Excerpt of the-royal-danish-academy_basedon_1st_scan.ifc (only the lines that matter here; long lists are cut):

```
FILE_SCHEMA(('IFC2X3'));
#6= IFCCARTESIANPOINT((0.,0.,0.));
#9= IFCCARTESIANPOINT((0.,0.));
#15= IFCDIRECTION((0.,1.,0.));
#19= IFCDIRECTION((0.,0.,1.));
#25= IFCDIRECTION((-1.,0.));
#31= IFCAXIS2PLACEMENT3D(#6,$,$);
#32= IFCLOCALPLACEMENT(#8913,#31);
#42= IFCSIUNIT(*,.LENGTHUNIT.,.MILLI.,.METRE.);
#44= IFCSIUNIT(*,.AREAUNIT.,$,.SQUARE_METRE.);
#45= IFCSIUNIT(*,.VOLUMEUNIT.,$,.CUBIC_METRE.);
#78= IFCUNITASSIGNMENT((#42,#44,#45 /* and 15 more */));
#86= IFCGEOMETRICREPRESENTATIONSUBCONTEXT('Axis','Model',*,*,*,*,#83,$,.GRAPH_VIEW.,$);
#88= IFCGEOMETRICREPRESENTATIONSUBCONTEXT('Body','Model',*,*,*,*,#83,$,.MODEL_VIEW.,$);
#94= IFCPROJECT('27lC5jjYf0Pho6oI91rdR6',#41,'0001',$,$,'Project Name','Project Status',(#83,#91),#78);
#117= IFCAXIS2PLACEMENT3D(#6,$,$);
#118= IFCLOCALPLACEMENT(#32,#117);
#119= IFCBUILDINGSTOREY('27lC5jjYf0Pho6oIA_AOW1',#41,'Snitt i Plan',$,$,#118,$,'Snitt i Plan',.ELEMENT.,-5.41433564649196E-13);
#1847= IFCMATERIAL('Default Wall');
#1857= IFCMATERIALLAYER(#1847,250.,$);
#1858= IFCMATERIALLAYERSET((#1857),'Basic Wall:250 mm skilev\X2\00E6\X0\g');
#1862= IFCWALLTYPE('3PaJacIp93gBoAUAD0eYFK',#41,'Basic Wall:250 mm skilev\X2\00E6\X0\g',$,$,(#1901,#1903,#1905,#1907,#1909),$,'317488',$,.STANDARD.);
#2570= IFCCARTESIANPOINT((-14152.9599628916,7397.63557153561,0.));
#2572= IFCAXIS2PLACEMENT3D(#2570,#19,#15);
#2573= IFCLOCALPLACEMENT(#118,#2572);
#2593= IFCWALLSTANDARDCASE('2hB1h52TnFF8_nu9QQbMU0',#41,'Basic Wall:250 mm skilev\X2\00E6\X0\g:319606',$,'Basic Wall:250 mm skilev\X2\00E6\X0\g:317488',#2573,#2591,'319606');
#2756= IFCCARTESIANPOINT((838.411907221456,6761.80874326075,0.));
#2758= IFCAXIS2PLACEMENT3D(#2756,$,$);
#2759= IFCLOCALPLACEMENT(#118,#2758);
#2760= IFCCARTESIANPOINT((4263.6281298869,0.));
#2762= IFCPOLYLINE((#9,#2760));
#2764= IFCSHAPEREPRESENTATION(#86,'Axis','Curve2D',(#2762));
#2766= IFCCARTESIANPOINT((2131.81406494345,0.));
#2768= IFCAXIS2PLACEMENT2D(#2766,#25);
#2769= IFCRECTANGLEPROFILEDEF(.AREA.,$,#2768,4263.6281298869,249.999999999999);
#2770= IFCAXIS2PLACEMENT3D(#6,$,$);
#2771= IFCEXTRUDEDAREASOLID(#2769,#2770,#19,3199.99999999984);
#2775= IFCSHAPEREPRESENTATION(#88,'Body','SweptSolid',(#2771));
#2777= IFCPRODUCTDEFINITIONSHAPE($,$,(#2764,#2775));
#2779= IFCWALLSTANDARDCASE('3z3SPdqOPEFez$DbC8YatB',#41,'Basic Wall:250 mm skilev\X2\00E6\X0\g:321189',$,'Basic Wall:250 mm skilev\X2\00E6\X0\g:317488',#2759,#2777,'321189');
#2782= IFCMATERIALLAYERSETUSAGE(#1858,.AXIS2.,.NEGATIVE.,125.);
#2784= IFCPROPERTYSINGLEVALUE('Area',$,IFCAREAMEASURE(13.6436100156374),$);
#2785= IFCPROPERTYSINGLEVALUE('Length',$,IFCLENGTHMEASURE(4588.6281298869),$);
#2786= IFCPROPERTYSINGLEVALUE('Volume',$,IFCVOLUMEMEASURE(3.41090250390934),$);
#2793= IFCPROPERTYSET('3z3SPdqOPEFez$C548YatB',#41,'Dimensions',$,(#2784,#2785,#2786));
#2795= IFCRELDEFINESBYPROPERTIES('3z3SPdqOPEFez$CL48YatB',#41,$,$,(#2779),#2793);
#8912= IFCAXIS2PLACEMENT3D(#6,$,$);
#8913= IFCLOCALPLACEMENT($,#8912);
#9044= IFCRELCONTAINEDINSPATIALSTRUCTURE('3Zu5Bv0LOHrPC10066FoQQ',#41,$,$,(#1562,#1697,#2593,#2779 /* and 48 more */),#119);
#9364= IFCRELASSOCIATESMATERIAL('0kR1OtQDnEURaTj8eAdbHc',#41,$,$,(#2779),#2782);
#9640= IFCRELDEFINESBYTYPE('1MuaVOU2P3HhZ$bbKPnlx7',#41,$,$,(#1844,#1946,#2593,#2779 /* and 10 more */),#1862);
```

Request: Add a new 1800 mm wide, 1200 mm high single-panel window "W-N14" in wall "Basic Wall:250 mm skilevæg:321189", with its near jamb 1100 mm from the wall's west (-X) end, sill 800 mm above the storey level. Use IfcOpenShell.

```python
import numpy as np
import ifcopenshell
import ifcopenshell.api.feature
import ifcopenshell.api.geometry
import ifcopenshell.api.pset
import ifcopenshell.api.root
import ifcopenshell.api.spatial
import ifcopenshell.api.type
import ifcopenshell.geom
import ifcopenshell.util.element
import ifcopenshell.util.placement
import ifcopenshell.util.representation
import ifcopenshell.util.shape
import ifcopenshell.util.unit

model = ifcopenshell.open("the-royal-danish-academy_basedon_1st_scan.ifc")
unit_scale = ifcopenshell.util.unit.calculate_unit_scale(model)
area_scale = ifcopenshell.util.unit.calculate_unit_scale(model, "AREAUNIT")
volume_scale = ifcopenshell.util.unit.calculate_unit_scale(model, "VOLUMEUNIT")
settings = ifcopenshell.geom.settings()


def volume(element):
    """Net volume in cubic metres, openings subtracted."""
    shape = ifcopenshell.geom.create_shape(settings, element)
    return ifcopenshell.util.shape.get_volume(shape.geometry)


wall = model.by_guid("3z3SPdqOPEFez$DbC8YatB")
storey = ifcopenshell.util.element.get_container(wall, ifc_class="IfcBuildingStorey")
context = ifcopenshell.util.representation.get_context(model, "Model", "Body", "MODEL_VIEW")
before = volume(wall)

width, height, from_end, sill = 1.8, 1.2, 1.1, 0.8  # metres

# The wall runs along its own X axis, and the end named is its -X end.
wall_shape = ifcopenshell.geom.create_shape(settings, wall)
x, y, z = ifcopenshell.util.shape.get_vertices(wall_shape.geometry).T
start = x.min() + from_end
face, thickness = float(y.min()), float(y.max() - y.min())
wall_matrix = ifcopenshell.util.placement.get_local_placement(wall.ObjectPlacement)
level = ifcopenshell.util.placement.get_local_placement(storey.ObjectPlacement)[2, 3]


def in_wall(x, y):
    """Placement at x, y metres in the wall's axes, at sill height."""
    matrix = wall_matrix.copy()
    matrix[:, 3] = wall_matrix @ np.array([x / unit_scale, y / unit_scale, 0.0, 1.0])
    matrix[2, 3] = level + sill / unit_scale
    return matrix


# Opening: a box that overshoots both wall faces by 50 mm.
opening = ifcopenshell.api.root.create_entity(model, ifc_class="IfcOpeningElement")
box = ifcopenshell.api.geometry.add_wall_representation(
    model, context=context, length=width, height=height, thickness=thickness + 0.1
)
ifcopenshell.api.geometry.assign_representation(model, product=opening, representation=box)
ifcopenshell.api.geometry.edit_object_placement(model, product=opening, matrix=in_wall(start, face - 0.05), is_si=False)
ifcopenshell.api.feature.add_feature(model, feature=opening, element=wall)

window = ifcopenshell.api.root.create_entity(model, ifc_class="IfcWindow", name="W-N14")
window.OverallWidth, window.OverallHeight = width / unit_scale, height / unit_scale
body = ifcopenshell.api.geometry.add_window_representation(
    model,
    context=context,
    overall_width=window.OverallWidth,
    overall_height=window.OverallHeight,
    partition_type="SINGLE_PANEL",
)
ifcopenshell.api.geometry.assign_representation(model, product=window, representation=body)
ifcopenshell.api.spatial.assign_container(model, products=[window], relating_structure=storey)
fills = ifcopenshell.api.feature.add_filling(model, opening=opening, element=window)
fills.OwnerHistory = window.OwnerHistory  # required in IFC2X3

# IFC2X3 keeps the operation on the window style.
style = ifcopenshell.api.root.create_entity(model, ifc_class="IfcWindowStyle", name="W-N14")
style.OperationType, style.ConstructionType = "SINGLE_PANEL", "NOTDEFINED"
style.ParameterTakesPrecedence = style.Sizeable = False
ifcopenshell.api.type.assign_type(model, related_objects=[window], relating_type=style)

# Centre the window in the wall's thickness.
ifcopenshell.api.geometry.edit_object_placement(model, product=window, matrix=in_wall(start, face), is_si=False)
window_shape = ifcopenshell.geom.create_shape(settings, window)
depth = ifcopenshell.util.shape.get_vertices(window_shape.geometry)[:, 1]
offset = face + thickness / 2 - (depth.min() + depth.max()) / 2
ifcopenshell.api.geometry.edit_object_placement(model, product=window, matrix=in_wall(start, offset), is_si=False)

after = volume(wall)

# Update the wall's stored quantities.
pset = model.by_id(ifcopenshell.util.element.get_pset(wall, "Dimensions", should_inherit=False)["id"])
ifcopenshell.api.pset.edit_pset(model, pset=pset, properties={
    "Area": model.create_entity("IfcAreaMeasure", after / thickness / area_scale),
    "Volume": model.create_entity("IfcVolumeMeasure", after / volume_scale),
})

print(f"wall volume {before:.3f} -> {after:.3f} m3")

model.write("the-royal-danish-academy_basedon_1st_scan_updated.ifc")
```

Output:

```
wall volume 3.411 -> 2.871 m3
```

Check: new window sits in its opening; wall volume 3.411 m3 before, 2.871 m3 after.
